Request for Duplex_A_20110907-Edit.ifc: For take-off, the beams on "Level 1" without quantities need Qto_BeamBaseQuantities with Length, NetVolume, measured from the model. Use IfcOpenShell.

First a look at what the model holds.

```python
import ifcopenshell
import ifcopenshell.util.element
import ifcopenshell.util.unit

model = ifcopenshell.open("Duplex_A_20110907-Edit.ifc")
print(model.schema)
for unit_type in ("LENGTHUNIT", "AREAUNIT", "VOLUMEUNIT"):
    print(unit_type, ifcopenshell.util.unit.calculate_unit_scale(model, unit_type))
storey = next(s for s in model.by_type("IfcBuildingStorey") if s.Name == "Level 1")
beams = [e for e in ifcopenshell.util.element.get_decomposition(storey) if e.is_a("IfcBeam")]
for e in sorted(beams, key=lambda e: e.id()):
    print(e.id(), e.is_a(), e.Name, list(ifcopenshell.util.element.get_psets(e, qtos_only=True)), sep=" | ")
```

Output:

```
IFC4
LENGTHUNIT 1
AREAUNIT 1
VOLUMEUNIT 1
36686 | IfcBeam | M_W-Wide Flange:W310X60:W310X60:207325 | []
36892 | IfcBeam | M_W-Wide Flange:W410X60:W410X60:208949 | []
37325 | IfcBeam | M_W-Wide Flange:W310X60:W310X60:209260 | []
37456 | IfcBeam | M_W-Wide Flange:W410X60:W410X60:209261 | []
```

```python
import ifcopenshell
import ifcopenshell.api.pset
import ifcopenshell.geom
import ifcopenshell.util.element
import ifcopenshell.util.shape
import ifcopenshell.util.unit

model = ifcopenshell.open("Duplex_A_20110907-Edit.ifc")
unit_scale = ifcopenshell.util.unit.calculate_unit_scale(model)
volume_scale = ifcopenshell.util.unit.calculate_unit_scale(model, "VOLUMEUNIT")
settings = ifcopenshell.geom.settings()

storey = next(s for s in model.by_type("IfcBuildingStorey") if s.Name == "Level 1")
beams = [e for e in ifcopenshell.util.element.get_decomposition(storey) if e.is_a("IfcBeam")]

for e in sorted(beams, key=lambda e: e.id()):
    if ifcopenshell.util.element.get_psets(e, qtos_only=True, should_inherit=False):
        continue
    # Geometry comes back in metres, in the element's own axes.
    shape = ifcopenshell.geom.create_shape(settings, e)
    values = {
        "Length": ifcopenshell.util.shape.get_max_xyz(shape.geometry) / unit_scale,
        "NetVolume": ifcopenshell.util.shape.get_volume(shape.geometry) / volume_scale,
    }
    qto = ifcopenshell.api.pset.add_qto(model, product=e, name="Qto_BeamBaseQuantities")
    ifcopenshell.api.pset.edit_qto(model, qto=qto, properties=values)
    print(e.id(), {k: round(v, 3) for k, v in values.items()})

model.write("Duplex_A_20110907-Edit_updated.ifc")
```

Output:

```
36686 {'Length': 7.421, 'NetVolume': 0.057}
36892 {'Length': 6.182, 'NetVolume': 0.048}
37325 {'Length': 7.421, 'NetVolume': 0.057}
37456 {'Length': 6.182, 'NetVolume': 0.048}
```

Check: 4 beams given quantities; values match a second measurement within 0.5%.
